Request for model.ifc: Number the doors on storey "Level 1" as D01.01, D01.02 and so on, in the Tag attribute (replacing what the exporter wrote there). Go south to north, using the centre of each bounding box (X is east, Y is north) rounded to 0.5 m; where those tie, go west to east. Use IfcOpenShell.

First a look at what the model holds.

```python
import ifcopenshell
import ifcopenshell.util.element
import ifcopenshell.util.placement

model = ifcopenshell.open("model.ifc")
print(model.schema)
storey = next(s for s in model.by_type("IfcBuildingStorey") if s.Name == "Level 1")
doors = [e for e in ifcopenshell.util.element.get_decomposition(storey) if e.is_a("IfcDoor")]
for e in sorted(doors, key=lambda e: e.id()):
    origin = ifcopenshell.util.placement.get_local_placement(e.ObjectPlacement)[:3, 3]
    print(e.id(), e.Tag, e.Name, origin.round(2) + 0.0, sep=" | ")
```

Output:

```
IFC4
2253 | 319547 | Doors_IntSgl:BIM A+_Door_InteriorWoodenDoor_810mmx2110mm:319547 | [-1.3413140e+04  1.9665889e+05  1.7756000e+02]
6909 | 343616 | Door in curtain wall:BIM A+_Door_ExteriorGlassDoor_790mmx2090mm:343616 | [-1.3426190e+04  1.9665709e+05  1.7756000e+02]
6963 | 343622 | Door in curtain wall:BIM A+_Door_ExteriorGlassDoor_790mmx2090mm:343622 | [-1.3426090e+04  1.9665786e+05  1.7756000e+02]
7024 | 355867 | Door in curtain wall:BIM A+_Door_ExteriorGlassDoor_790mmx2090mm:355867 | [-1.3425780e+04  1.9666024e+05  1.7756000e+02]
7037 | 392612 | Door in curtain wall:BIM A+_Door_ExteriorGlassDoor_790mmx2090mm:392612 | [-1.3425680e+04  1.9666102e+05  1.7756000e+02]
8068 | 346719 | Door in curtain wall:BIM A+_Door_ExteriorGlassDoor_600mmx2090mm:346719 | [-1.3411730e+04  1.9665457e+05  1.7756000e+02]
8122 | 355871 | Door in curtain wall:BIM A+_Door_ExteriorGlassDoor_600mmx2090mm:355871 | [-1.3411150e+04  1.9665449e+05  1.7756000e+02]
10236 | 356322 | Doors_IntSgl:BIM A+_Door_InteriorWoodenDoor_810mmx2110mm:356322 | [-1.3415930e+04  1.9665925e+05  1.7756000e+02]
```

```python
import ifcopenshell
import ifcopenshell.geom
import ifcopenshell.util.element
import ifcopenshell.util.shape

model = ifcopenshell.open("model.ifc")
settings = ifcopenshell.geom.settings()
settings.set("use-world-coords", True)


def centre(element):
    shape = ifcopenshell.geom.create_shape(settings, element)
    return ifcopenshell.util.shape.get_bbox_centroid(shape.geometry)


storey = next(s for s in model.by_type("IfcBuildingStorey") if s.Name == "Level 1")
doors = [e for e in ifcopenshell.util.element.get_decomposition(storey) if e.is_a("IfcDoor")]

# Insertion points can sit at a corner or the storey origin, so sort by the geometry (in metres).
centres = {e: centre(e) for e in doors}
doors.sort(key=lambda e: (round(centres[e][1] / 0.5), centres[e][0]))

for i, e in enumerate(doors, start=1):
    number = f"D01.{i:02d}"
    e.Tag = number
    print(e.id(), number)

model.write("model_edited.ifc")
```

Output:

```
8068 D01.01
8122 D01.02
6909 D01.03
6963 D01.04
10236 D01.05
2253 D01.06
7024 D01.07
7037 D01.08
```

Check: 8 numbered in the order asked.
